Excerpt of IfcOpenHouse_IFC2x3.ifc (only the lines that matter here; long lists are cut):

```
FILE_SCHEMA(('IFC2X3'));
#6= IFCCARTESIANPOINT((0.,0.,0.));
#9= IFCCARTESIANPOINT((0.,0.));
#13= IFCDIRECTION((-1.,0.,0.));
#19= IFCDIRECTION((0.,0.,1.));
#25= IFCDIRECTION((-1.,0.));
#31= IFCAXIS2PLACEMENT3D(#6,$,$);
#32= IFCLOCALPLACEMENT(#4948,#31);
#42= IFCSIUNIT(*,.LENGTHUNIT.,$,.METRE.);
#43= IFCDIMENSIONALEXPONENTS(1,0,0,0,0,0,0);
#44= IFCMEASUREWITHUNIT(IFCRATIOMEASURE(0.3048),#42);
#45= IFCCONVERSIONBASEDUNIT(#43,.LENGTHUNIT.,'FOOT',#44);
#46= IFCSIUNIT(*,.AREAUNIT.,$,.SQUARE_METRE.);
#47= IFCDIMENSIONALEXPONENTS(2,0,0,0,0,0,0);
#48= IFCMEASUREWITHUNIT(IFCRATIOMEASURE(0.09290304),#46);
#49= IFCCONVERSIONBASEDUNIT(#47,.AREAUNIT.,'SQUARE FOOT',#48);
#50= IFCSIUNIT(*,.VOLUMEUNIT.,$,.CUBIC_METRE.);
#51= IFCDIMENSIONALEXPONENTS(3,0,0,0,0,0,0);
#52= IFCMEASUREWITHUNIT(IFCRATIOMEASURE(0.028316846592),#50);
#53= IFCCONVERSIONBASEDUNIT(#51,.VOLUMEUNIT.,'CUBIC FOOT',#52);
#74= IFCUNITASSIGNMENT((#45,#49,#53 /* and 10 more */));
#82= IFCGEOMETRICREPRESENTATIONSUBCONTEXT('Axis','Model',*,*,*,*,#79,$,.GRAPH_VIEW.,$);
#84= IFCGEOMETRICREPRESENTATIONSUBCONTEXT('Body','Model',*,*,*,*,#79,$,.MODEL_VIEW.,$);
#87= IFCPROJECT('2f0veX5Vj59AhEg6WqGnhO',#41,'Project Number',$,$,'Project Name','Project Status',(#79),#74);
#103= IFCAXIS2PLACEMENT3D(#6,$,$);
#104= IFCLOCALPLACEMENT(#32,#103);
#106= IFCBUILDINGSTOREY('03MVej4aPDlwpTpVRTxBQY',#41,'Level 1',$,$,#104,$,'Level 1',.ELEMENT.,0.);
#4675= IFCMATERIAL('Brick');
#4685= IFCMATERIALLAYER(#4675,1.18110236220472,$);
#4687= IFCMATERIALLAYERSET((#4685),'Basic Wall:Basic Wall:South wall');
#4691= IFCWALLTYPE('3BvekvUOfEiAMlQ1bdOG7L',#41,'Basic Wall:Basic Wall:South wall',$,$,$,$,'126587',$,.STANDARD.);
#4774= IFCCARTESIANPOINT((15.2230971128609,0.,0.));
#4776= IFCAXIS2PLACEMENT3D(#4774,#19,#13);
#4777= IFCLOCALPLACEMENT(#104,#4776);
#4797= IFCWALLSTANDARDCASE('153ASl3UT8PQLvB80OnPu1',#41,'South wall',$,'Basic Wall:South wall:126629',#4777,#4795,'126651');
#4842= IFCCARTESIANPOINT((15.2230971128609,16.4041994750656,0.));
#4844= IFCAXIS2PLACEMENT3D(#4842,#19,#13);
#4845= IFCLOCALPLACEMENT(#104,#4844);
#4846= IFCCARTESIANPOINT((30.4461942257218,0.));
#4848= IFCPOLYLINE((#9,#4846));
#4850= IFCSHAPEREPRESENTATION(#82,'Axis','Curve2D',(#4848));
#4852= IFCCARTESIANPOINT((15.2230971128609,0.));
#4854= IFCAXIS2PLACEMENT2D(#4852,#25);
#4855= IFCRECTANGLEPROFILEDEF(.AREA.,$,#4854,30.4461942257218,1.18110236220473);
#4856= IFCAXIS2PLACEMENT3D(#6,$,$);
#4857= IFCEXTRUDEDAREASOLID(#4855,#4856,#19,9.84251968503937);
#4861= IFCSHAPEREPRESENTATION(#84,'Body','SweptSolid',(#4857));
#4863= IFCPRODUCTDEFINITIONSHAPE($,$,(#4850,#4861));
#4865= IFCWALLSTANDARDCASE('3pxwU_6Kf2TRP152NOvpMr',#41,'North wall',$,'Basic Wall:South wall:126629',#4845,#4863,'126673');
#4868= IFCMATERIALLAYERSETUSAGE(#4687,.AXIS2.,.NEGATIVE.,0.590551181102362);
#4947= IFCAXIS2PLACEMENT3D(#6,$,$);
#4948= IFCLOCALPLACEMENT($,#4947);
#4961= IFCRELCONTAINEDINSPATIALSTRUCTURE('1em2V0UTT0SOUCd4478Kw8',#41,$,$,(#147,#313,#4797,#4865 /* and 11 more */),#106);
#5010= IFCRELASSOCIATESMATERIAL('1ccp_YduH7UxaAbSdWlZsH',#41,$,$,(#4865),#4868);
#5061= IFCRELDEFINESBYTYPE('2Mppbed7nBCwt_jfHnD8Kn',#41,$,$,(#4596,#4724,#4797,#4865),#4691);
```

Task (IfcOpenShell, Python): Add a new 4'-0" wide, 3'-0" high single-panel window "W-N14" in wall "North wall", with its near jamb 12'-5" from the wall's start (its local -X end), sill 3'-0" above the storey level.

```python
import numpy as np
import ifcopenshell
import ifcopenshell.api.feature
import ifcopenshell.api.geometry
import ifcopenshell.api.root
import ifcopenshell.api.spatial
import ifcopenshell.api.type
import ifcopenshell.geom
import ifcopenshell.util.element
import ifcopenshell.util.placement
import ifcopenshell.util.representation
import ifcopenshell.util.shape
import ifcopenshell.util.unit

model = ifcopenshell.open("IfcOpenHouse_IFC2x3.ifc")
unit_scale = ifcopenshell.util.unit.calculate_unit_scale(model)
settings = ifcopenshell.geom.settings()


def volume(element):
    """Net volume in cubic metres, openings subtracted."""
    shape = ifcopenshell.geom.create_shape(settings, element)
    return ifcopenshell.util.shape.get_volume(shape.geometry)


wall = model.by_guid("3pxwU_6Kf2TRP152NOvpMr")
storey = ifcopenshell.util.element.get_container(wall, ifc_class="IfcBuildingStorey")
context = ifcopenshell.util.representation.get_context(model, "Model", "Body", "MODEL_VIEW")
before = volume(wall)

width, height, from_end, sill = 1.2192, 0.9144, 3.7846, 0.9144  # metres

# The wall runs along its own X axis, and the end named is its -X end.
wall_shape = ifcopenshell.geom.create_shape(settings, wall)
x, y, z = ifcopenshell.util.shape.get_vertices(wall_shape.geometry).T
start = x.min() + from_end
face, thickness = float(y.min()), float(y.max() - y.min())
wall_matrix = ifcopenshell.util.placement.get_local_placement(wall.ObjectPlacement)
level = ifcopenshell.util.placement.get_local_placement(storey.ObjectPlacement)[2, 3]


def in_wall(x, y):
    """Placement at x, y metres in the wall's axes, at sill height."""
    matrix = wall_matrix.copy()
    matrix[:, 3] = wall_matrix @ np.array([x / unit_scale, y / unit_scale, 0.0, 1.0])
    matrix[2, 3] = level + sill / unit_scale
    return matrix


# Opening: a box that overshoots both wall faces by 50 mm.
opening = ifcopenshell.api.root.create_entity(model, ifc_class="IfcOpeningElement")
box = ifcopenshell.api.geometry.add_wall_representation(
    model, context=context, length=width, height=height, thickness=thickness + 0.1
)
ifcopenshell.api.geometry.assign_representation(model, product=opening, representation=box)
ifcopenshell.api.geometry.edit_object_placement(model, product=opening, matrix=in_wall(start, face - 0.05), is_si=False)
ifcopenshell.api.feature.add_feature(model, feature=opening, element=wall)

window = ifcopenshell.api.root.create_entity(model, ifc_class="IfcWindow", name="W-N14")
window.OverallWidth, window.OverallHeight = width / unit_scale, height / unit_scale
body = ifcopenshell.api.geometry.add_window_representation(
    model,
    context=context,
    overall_width=window.OverallWidth,
    overall_height=window.OverallHeight,
    partition_type="SINGLE_PANEL",
)
ifcopenshell.api.geometry.assign_representation(model, product=window, representation=body)
ifcopenshell.api.spatial.assign_container(model, products=[window], relating_structure=storey)
fills = ifcopenshell.api.feature.add_filling(model, opening=opening, element=window)
fills.OwnerHistory = window.OwnerHistory  # required in IFC2X3

# IFC2X3 keeps the operation on the window style.
style = ifcopenshell.api.root.create_entity(model, ifc_class="IfcWindowStyle", name="W-N14")
style.OperationType, style.ConstructionType = "SINGLE_PANEL", "NOTDEFINED"
style.ParameterTakesPrecedence = style.Sizeable = False
ifcopenshell.api.type.assign_type(model, related_objects=[window], relating_type=style)

# Centre the window in the wall's thickness.
ifcopenshell.api.geometry.edit_object_placement(model, product=window, matrix=in_wall(start, face), is_si=False)
window_shape = ifcopenshell.geom.create_shape(settings, window)
depth = ifcopenshell.util.shape.get_vertices(window_shape.geometry)[:, 1]
offset = face + thickness / 2 - (depth.min() + depth.max()) / 2
ifcopenshell.api.geometry.edit_object_placement(model, product=window, matrix=in_wall(start, offset), is_si=False)

after = volume(wall)

print(f"wall volume {before:.3f} -> {after:.3f} m3")

model.write("IfcOpenHouse_IFC2x3_edited.ifc")
```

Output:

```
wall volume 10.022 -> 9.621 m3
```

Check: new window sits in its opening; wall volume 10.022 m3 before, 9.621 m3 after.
